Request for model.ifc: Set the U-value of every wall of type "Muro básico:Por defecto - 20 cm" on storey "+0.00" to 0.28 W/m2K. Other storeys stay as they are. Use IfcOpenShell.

First a look at what the model holds.

```python
import ifcopenshell
import ifcopenshell.util.element

model = ifcopenshell.open("model.ifc")
print(model.schema)
storey = next(s for s in model.by_type("IfcBuildingStorey") if s.Name == "+0.00")
walls = [e for e in ifcopenshell.util.element.get_decomposition(storey) if e.is_a("IfcWall")]
seen = {}
for e in walls:
    element_type = ifcopenshell.util.element.get_type(e)
    key = (element_type.Name if element_type != e and element_type else None, ifcopenshell.util.element.get_pset(e, "Pset_WallCommon", "ThermalTransmittance"))
    seen[key] = seen.get(key, 0) + 1
for (name, value), count in sorted(seen.items(), key=str):
    print(count, "x", name, "|", value)
```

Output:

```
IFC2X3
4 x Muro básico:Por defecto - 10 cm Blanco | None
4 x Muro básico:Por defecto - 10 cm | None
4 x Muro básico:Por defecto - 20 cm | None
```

```python
import ifcopenshell
import ifcopenshell.api.pset
import ifcopenshell.util.element

model = ifcopenshell.open("model.ifc")

storey = next(s for s in model.by_type("IfcBuildingStorey") if s.Name == "+0.00")
walls = [e for e in ifcopenshell.util.element.get_decomposition(storey) if e.is_a("IfcWall")]

count = 0
for e in walls:
    element_type = ifcopenshell.util.element.get_type(e)
    if element_type in (None, e) or element_type.Name != "Muro básico:Por defecto - 20 cm":
        continue
    # add_pset returns the element's existing set when there is one.
    pset = ifcopenshell.api.pset.add_pset(model, product=e, name="Pset_WallCommon")
    ifcopenshell.api.pset.edit_pset(model, pset=pset, properties={"ThermalTransmittance": 0.28})
    count += 1

print(count, "walls updated")

model.write("model_updated.ifc")
```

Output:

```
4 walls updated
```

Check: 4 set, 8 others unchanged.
